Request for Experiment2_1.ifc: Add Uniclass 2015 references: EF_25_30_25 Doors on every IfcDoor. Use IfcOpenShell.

First a look at what the model holds.

```python
import ifcopenshell

model = ifcopenshell.open("Experiment2_1.ifc")
print(model.schema)
print("classifications:", [c.Name for c in model.by_type("IfcClassification")])
for ifc_class in ("IfcDoor", "IfcRoof", "IfcStair", "IfcWall", "IfcWindow"):
    print(ifc_class, len(model.by_type(ifc_class)))
```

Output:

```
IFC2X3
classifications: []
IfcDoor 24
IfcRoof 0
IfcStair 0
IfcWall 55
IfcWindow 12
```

```python
import ifcopenshell
import ifcopenshell.api.classification

model = ifcopenshell.open("Experiment2_1.ifc")

# IFC2X3 requires Source and Edition and has no link from the project to the system.
system = model.create_entity("IfcClassification", Source="NBS", Edition="2015", Name="Uniclass 2015")

codes = {
    "IfcDoor": ("EF_25_30_25", "Doors"),
}
for ifc_class, (code, name) in codes.items():
    products = model.by_type(ifc_class)
    ifcopenshell.api.classification.add_reference(
        model, products=products, classification=system, identification=code, name=name
    )
    print(code, len(products))

model.write("Experiment2_1_v2.ifc")
```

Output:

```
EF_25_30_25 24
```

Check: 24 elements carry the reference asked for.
